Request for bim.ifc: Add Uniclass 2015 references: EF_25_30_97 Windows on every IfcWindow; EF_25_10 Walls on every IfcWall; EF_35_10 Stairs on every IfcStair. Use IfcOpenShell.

First a look at what the model holds.

```python
import ifcopenshell

model = ifcopenshell.open("bim.ifc")
print(model.schema)
print("classifications:", [c.Name for c in model.by_type("IfcClassification")])
for ifc_class in ("IfcDoor", "IfcRoof", "IfcStair", "IfcWall", "IfcWindow"):
    print(ifc_class, len(model.by_type(ifc_class)))
```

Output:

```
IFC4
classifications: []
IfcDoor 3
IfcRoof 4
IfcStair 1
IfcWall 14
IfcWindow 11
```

```python
import ifcopenshell
import ifcopenshell.api.classification

model = ifcopenshell.open("bim.ifc")

system = ifcopenshell.api.classification.add_classification(model, classification="Uniclass 2015")

codes = {
    "IfcWindow": ("EF_25_30_97", "Windows"),
    "IfcWall": ("EF_25_10", "Walls"),
    "IfcStair": ("EF_35_10", "Stairs"),
}
for ifc_class, (code, name) in codes.items():
    products = model.by_type(ifc_class)
    ifcopenshell.api.classification.add_reference(
        model, products=products, classification=system, identification=code, name=name
    )
    print(code, len(products))

model.write("bim_rev.ifc")
```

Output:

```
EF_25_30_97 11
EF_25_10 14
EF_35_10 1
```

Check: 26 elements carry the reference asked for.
